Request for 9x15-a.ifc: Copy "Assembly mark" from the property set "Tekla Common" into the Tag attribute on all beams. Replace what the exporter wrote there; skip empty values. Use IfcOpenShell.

First a look at what the model holds.

```python
import ifcopenshell
import ifcopenshell.util.element

model = ifcopenshell.open("9x15-a.ifc")
print(model.schema)
beams = model.by_type("IfcBeam")
print(len(beams), "beams")
for e in beams[:8]:
    source = ifcopenshell.util.element.get_pset(e, "Tekla Common", "Assembly mark")
    target = e.Tag
    print(e.id(), repr(source), repr(target), sep=" | ")
```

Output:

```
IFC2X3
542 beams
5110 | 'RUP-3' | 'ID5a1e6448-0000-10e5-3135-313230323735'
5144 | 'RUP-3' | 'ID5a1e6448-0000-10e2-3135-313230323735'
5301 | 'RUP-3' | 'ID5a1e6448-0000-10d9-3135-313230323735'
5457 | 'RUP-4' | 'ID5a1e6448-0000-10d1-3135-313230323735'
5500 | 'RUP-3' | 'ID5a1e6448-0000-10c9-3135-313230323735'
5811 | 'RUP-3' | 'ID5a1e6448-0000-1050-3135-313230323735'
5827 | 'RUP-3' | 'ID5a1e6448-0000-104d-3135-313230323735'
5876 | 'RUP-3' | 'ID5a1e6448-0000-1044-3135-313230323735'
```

```python
import ifcopenshell
import ifcopenshell.util.element

model = ifcopenshell.open("9x15-a.ifc")

count = 0
for e in model.by_type("IfcBeam"):
    value = ifcopenshell.util.element.get_pset(e, "Tekla Common", "Assembly mark")
    current = e.Tag
    if not value or not value.strip() or current == value:
        continue
    e.Tag = value
    count += 1

print(count, "beams updated")

model.write("9x15-a_edited.ifc")
```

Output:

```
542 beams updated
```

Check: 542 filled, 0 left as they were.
